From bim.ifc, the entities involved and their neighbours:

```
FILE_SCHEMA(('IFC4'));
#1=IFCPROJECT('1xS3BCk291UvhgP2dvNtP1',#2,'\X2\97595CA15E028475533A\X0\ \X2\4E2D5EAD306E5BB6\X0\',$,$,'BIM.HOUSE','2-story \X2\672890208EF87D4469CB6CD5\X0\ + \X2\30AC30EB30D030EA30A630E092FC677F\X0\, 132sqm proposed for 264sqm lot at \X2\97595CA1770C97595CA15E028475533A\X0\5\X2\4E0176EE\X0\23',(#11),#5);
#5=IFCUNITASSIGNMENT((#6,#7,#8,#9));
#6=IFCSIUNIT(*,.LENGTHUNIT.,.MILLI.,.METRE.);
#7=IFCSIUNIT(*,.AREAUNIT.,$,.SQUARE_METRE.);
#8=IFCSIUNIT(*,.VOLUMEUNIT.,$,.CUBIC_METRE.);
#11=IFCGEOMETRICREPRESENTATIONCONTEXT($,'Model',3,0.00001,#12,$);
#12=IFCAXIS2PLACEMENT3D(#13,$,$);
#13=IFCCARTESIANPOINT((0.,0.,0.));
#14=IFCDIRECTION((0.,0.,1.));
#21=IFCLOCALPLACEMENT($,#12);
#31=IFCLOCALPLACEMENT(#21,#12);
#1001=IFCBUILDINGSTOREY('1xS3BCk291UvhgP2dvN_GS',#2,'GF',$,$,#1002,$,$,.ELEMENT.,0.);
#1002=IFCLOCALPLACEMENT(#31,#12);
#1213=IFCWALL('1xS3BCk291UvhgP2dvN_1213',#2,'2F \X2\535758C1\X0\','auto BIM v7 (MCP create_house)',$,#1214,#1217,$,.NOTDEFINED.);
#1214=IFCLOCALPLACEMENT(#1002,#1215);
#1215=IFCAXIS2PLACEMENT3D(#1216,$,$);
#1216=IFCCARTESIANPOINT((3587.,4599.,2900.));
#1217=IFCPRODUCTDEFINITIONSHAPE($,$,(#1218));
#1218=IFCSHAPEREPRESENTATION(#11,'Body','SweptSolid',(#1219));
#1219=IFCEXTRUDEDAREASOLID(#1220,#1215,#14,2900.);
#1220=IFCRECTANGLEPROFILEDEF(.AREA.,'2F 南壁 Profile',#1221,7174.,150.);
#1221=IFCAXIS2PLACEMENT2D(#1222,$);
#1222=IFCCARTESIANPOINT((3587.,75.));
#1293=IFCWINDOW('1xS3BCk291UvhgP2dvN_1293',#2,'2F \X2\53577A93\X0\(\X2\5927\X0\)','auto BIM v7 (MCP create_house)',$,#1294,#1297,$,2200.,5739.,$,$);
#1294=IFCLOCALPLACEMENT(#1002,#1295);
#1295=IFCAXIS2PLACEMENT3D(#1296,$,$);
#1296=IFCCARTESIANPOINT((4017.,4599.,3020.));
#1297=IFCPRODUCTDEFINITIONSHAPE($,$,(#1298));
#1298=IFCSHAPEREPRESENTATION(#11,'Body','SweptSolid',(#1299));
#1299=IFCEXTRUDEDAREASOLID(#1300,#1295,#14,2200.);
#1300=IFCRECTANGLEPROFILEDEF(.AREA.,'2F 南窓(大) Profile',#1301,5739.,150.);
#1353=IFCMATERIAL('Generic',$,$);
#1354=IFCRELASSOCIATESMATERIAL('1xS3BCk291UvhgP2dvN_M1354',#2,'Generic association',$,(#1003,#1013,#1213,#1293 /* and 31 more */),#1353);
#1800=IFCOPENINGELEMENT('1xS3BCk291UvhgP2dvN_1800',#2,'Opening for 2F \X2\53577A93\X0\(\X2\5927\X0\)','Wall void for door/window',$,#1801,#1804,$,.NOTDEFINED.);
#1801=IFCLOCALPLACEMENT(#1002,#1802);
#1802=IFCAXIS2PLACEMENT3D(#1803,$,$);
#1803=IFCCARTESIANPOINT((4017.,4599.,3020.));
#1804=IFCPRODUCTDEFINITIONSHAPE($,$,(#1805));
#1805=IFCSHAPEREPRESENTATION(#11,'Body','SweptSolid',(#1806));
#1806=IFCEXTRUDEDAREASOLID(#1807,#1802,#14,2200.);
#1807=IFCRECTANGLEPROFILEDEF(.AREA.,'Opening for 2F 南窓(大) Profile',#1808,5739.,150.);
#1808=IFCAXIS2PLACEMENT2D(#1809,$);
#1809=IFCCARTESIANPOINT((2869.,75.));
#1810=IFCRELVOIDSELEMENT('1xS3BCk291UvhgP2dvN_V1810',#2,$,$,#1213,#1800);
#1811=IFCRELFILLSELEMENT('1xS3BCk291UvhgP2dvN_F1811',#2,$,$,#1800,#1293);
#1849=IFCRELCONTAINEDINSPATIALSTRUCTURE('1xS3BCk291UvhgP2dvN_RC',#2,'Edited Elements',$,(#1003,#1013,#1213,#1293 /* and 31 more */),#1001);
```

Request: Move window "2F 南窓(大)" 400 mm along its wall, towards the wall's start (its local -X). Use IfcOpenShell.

```python
import ifcopenshell
import ifcopenshell.api.geometry
import ifcopenshell.util.placement
import ifcopenshell.util.unit

model = ifcopenshell.open("bim.ifc")
unit_scale = ifcopenshell.util.unit.calculate_unit_scale(model)

window = model.by_id(1293)
opening = window.FillsVoids[0].RelatingOpeningElement
wall = opening.VoidsElements[0].RelatingBuildingElement

wall_matrix = ifcopenshell.util.placement.get_local_placement(wall.ObjectPlacement)
shift = wall_matrix[:3, 0] * -0.4 / unit_scale
before = ifcopenshell.util.placement.get_local_placement(window.ObjectPlacement)[:3, 3].copy()

# The window is not placed relative to its opening, so move both.
for product in (opening, window):
    matrix = ifcopenshell.util.placement.get_local_placement(product.ObjectPlacement)
    matrix[:3, 3] += shift
    ifcopenshell.api.geometry.edit_object_placement(model, product=product, matrix=matrix, is_si=False)

after = ifcopenshell.util.placement.get_local_placement(window.ObjectPlacement)[:3, 3]
print("window moved by", (after - before).round(3) + 0.0)

model.write("bim_rev.ifc")
```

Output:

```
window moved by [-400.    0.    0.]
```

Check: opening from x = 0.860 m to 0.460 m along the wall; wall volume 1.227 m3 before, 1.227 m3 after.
